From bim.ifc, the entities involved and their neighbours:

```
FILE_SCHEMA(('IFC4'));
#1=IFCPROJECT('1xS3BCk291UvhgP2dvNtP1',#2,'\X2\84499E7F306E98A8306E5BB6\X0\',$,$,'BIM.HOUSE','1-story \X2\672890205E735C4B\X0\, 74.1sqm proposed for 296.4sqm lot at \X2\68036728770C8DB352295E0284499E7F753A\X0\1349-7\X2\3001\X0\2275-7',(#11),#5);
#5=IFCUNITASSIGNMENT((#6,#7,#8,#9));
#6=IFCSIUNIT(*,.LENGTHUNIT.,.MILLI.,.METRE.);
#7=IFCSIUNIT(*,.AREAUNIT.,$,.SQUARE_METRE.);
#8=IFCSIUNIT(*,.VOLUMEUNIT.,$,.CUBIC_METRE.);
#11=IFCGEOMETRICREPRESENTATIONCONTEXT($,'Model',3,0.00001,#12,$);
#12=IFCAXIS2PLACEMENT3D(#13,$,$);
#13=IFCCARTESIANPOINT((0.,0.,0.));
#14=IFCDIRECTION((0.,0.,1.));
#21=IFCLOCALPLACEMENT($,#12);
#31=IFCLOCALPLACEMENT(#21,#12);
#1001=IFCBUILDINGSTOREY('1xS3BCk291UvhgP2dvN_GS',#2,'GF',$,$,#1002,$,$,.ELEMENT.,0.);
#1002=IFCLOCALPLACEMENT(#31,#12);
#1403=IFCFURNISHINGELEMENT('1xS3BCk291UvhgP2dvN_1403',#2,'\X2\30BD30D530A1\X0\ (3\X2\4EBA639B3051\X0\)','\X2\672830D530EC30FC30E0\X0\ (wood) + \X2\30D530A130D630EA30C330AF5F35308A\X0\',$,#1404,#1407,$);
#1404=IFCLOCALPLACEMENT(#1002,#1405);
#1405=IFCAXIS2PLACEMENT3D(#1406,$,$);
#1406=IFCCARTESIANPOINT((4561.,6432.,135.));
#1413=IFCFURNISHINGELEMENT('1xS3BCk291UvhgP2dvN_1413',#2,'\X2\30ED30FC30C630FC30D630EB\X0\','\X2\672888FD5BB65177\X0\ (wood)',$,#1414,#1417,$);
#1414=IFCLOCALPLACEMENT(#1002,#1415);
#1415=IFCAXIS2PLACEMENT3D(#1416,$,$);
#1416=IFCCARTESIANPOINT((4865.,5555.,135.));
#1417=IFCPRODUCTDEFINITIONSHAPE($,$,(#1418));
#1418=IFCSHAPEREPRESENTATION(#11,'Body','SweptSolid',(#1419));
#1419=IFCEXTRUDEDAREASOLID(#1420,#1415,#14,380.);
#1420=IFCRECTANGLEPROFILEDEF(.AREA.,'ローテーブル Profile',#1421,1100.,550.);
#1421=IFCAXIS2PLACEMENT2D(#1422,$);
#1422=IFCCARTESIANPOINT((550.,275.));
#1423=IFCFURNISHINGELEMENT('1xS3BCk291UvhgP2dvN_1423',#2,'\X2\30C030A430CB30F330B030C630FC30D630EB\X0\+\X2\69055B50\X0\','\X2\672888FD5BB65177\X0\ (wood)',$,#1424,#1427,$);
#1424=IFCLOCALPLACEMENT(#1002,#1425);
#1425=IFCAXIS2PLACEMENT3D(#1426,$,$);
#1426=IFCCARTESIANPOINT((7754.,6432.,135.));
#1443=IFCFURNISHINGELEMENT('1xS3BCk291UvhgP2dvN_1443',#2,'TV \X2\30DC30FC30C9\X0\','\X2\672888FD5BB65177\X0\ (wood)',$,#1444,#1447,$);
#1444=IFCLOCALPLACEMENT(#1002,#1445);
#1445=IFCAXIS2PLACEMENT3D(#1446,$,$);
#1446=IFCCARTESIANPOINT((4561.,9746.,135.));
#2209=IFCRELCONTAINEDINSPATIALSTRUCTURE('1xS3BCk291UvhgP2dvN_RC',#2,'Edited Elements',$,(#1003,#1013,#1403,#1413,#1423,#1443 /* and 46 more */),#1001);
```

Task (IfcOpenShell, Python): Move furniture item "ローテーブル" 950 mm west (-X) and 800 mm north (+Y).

```python
import ifcopenshell
import ifcopenshell.api.geometry
import ifcopenshell.util.placement
import ifcopenshell.util.unit

model = ifcopenshell.open("bim.ifc")
unit_scale = ifcopenshell.util.unit.calculate_unit_scale(model)

item = model.by_guid("1xS3BCk291UvhgP2dvN_1413")
matrix = ifcopenshell.util.placement.get_local_placement(item.ObjectPlacement)
matrix[0, 3] -= 0.95 / unit_scale
matrix[1, 3] += 0.8 / unit_scale
ifcopenshell.api.geometry.edit_object_placement(model, product=item, matrix=matrix, is_si=False)

print(ifcopenshell.util.placement.get_local_placement(item.ObjectPlacement).round(3) + 0.0)

model.write("bim_v2.ifc")
```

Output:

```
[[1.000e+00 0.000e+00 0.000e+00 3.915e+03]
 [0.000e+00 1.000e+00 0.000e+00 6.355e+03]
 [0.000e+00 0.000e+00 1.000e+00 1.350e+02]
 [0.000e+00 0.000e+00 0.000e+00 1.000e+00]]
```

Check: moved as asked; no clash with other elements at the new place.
